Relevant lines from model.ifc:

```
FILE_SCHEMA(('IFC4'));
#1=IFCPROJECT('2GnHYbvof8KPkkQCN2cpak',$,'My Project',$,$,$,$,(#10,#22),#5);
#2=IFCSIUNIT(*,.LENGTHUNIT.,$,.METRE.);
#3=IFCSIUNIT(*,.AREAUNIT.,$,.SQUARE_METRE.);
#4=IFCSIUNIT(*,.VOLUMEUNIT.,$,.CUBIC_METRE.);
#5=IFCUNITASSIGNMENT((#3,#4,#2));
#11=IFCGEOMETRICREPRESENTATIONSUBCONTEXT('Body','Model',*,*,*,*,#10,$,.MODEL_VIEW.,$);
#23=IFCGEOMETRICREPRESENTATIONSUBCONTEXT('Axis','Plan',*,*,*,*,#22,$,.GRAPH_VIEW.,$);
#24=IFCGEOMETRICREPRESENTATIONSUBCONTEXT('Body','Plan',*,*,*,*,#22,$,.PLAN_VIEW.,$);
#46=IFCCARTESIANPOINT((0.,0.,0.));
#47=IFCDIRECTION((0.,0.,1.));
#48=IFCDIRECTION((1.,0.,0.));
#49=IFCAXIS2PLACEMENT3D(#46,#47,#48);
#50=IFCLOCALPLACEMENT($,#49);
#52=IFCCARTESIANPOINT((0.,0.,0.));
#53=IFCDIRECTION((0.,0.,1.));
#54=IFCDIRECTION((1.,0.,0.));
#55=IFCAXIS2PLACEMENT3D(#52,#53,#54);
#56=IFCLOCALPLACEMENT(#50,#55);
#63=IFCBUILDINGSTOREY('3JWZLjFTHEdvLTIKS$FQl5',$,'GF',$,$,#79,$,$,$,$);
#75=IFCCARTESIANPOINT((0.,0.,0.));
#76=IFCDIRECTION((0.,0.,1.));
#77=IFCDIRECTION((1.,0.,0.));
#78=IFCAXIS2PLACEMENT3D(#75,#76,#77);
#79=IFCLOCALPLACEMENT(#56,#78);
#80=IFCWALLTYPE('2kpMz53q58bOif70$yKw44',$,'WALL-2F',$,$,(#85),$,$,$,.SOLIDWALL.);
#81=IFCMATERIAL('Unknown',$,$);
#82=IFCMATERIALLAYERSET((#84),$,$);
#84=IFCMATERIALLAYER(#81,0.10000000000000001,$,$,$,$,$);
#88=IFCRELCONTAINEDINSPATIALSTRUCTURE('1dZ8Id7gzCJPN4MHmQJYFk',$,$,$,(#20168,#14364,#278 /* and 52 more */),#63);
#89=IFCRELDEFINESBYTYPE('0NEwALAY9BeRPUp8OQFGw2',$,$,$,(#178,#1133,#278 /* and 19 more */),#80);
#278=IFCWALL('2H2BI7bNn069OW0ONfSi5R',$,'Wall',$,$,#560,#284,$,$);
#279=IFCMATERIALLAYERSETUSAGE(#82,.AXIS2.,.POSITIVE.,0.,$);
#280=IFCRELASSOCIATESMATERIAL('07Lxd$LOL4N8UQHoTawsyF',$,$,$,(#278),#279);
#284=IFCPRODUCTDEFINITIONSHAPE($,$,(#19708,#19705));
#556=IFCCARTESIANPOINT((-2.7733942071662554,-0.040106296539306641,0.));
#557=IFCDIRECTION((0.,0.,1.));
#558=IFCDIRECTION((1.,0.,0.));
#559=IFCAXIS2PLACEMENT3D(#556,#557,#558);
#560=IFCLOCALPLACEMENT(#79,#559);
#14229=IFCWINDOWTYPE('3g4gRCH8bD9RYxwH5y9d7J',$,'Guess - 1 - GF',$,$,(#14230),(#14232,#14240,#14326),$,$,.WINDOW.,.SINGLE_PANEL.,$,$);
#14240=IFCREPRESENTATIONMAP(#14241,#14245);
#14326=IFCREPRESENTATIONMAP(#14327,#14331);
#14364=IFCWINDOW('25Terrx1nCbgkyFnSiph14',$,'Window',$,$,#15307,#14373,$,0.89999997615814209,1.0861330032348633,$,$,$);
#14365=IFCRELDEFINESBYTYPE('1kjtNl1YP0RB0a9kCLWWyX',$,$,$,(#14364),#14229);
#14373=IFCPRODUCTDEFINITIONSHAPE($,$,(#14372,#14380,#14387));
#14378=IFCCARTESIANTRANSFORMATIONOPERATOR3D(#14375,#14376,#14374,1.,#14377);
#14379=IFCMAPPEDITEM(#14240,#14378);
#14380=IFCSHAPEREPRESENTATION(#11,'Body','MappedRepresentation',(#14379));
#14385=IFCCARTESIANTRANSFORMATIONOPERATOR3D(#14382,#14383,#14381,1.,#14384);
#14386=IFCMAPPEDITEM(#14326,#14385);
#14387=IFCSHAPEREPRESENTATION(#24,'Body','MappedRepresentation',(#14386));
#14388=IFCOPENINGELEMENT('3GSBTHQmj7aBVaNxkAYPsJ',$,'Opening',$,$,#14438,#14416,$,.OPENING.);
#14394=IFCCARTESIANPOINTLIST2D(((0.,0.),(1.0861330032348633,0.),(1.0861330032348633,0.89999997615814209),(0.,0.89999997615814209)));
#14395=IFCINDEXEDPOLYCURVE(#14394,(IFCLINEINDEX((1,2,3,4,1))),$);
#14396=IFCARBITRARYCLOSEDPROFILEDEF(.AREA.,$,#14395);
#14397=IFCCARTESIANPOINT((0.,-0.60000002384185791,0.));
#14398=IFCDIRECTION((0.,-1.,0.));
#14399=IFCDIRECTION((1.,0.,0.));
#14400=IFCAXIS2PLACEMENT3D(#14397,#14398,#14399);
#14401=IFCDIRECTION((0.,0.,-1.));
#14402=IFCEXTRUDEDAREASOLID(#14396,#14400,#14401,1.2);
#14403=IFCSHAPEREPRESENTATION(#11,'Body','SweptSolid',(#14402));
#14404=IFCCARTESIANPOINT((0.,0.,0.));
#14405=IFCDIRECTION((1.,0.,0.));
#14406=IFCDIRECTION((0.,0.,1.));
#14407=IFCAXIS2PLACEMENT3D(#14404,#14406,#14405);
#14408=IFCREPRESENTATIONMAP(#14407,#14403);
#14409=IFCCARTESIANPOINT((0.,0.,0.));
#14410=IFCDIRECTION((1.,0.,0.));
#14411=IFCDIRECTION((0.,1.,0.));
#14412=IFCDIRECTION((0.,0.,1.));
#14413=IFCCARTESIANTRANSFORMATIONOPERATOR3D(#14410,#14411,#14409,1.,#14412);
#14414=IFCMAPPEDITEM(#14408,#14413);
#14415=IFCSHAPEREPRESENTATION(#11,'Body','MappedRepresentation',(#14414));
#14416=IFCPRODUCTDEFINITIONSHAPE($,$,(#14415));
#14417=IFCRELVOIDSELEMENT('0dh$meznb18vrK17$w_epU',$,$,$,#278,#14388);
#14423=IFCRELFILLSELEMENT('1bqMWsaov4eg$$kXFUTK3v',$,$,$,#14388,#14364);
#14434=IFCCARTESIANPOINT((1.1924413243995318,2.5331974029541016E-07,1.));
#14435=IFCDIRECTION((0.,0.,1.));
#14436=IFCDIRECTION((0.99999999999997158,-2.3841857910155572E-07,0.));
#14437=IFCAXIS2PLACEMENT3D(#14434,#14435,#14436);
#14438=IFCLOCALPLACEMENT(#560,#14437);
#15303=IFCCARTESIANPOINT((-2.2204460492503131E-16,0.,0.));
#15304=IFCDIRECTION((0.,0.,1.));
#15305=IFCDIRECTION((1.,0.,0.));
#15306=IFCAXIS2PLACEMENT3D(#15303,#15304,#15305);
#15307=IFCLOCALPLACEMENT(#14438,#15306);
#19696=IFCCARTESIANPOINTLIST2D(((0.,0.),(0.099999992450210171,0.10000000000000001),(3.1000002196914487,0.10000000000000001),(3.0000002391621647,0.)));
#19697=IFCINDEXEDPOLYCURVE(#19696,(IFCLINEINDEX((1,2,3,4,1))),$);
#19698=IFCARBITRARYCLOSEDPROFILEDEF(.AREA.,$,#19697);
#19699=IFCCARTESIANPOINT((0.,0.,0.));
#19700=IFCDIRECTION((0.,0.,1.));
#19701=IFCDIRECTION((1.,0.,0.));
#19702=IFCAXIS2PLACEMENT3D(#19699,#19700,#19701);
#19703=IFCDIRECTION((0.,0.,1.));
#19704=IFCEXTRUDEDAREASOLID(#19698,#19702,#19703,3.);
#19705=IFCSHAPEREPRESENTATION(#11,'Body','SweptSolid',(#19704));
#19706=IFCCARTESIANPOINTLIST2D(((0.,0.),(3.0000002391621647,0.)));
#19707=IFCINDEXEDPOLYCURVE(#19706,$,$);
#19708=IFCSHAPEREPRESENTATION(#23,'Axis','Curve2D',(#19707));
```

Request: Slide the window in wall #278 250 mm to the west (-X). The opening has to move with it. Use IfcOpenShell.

```python
import ifcopenshell
import ifcopenshell.api.geometry
import ifcopenshell.util.placement

model = ifcopenshell.open("model.ifc")

window = model.by_id(14364)
opening = window.FillsVoids[0].RelatingOpeningElement
wall = opening.VoidsElements[0].RelatingBuildingElement

wall_matrix = ifcopenshell.util.placement.get_local_placement(wall.ObjectPlacement)
shift = wall_matrix[:3, 0] * -0.25
before = ifcopenshell.util.placement.get_local_placement(window.ObjectPlacement)[:3, 3].copy()

# The window is placed relative to its opening, so it follows when the opening moves.
matrix = ifcopenshell.util.placement.get_local_placement(opening.ObjectPlacement)
matrix[:3, 3] += shift
ifcopenshell.api.geometry.edit_object_placement(
    model, product=opening, matrix=matrix, is_si=False, should_transform_children=True
)

after = ifcopenshell.util.placement.get_local_placement(window.ObjectPlacement)[:3, 3]
print("window moved by", (after - before).round(3) + 0.0)

model.write("model_edited.ifc")
```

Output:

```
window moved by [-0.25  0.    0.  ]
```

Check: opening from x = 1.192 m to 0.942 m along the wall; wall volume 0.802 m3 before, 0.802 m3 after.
